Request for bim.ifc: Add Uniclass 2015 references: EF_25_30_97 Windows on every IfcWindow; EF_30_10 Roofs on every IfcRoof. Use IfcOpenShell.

First a look at what the model holds.

```python
import ifcopenshell

model = ifcopenshell.open("bim.ifc")
print(model.schema)
print("classifications:", [c.Name for c in model.by_type("IfcClassification")])
for ifc_class in ("IfcDoor", "IfcRoof", "IfcStair", "IfcWall", "IfcWindow"):
    print(ifc_class, len(model.by_type(ifc_class)))
```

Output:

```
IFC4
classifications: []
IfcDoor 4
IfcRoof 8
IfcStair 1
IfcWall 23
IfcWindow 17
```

```python
import ifcopenshell
import ifcopenshell.api.classification

model = ifcopenshell.open("bim.ifc")

system = ifcopenshell.api.classification.add_classification(model, classification="Uniclass 2015")

codes = {
    "IfcWindow": ("EF_25_30_97", "Windows"),
    "IfcRoof": ("EF_30_10", "Roofs"),
}
for ifc_class, (code, name) in codes.items():
    products = model.by_type(ifc_class)
    ifcopenshell.api.classification.add_reference(
        model, products=products, classification=system, identification=code, name=name
    )
    print(code, len(products))

model.write("bim-out.ifc")
```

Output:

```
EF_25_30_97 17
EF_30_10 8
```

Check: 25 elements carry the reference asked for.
